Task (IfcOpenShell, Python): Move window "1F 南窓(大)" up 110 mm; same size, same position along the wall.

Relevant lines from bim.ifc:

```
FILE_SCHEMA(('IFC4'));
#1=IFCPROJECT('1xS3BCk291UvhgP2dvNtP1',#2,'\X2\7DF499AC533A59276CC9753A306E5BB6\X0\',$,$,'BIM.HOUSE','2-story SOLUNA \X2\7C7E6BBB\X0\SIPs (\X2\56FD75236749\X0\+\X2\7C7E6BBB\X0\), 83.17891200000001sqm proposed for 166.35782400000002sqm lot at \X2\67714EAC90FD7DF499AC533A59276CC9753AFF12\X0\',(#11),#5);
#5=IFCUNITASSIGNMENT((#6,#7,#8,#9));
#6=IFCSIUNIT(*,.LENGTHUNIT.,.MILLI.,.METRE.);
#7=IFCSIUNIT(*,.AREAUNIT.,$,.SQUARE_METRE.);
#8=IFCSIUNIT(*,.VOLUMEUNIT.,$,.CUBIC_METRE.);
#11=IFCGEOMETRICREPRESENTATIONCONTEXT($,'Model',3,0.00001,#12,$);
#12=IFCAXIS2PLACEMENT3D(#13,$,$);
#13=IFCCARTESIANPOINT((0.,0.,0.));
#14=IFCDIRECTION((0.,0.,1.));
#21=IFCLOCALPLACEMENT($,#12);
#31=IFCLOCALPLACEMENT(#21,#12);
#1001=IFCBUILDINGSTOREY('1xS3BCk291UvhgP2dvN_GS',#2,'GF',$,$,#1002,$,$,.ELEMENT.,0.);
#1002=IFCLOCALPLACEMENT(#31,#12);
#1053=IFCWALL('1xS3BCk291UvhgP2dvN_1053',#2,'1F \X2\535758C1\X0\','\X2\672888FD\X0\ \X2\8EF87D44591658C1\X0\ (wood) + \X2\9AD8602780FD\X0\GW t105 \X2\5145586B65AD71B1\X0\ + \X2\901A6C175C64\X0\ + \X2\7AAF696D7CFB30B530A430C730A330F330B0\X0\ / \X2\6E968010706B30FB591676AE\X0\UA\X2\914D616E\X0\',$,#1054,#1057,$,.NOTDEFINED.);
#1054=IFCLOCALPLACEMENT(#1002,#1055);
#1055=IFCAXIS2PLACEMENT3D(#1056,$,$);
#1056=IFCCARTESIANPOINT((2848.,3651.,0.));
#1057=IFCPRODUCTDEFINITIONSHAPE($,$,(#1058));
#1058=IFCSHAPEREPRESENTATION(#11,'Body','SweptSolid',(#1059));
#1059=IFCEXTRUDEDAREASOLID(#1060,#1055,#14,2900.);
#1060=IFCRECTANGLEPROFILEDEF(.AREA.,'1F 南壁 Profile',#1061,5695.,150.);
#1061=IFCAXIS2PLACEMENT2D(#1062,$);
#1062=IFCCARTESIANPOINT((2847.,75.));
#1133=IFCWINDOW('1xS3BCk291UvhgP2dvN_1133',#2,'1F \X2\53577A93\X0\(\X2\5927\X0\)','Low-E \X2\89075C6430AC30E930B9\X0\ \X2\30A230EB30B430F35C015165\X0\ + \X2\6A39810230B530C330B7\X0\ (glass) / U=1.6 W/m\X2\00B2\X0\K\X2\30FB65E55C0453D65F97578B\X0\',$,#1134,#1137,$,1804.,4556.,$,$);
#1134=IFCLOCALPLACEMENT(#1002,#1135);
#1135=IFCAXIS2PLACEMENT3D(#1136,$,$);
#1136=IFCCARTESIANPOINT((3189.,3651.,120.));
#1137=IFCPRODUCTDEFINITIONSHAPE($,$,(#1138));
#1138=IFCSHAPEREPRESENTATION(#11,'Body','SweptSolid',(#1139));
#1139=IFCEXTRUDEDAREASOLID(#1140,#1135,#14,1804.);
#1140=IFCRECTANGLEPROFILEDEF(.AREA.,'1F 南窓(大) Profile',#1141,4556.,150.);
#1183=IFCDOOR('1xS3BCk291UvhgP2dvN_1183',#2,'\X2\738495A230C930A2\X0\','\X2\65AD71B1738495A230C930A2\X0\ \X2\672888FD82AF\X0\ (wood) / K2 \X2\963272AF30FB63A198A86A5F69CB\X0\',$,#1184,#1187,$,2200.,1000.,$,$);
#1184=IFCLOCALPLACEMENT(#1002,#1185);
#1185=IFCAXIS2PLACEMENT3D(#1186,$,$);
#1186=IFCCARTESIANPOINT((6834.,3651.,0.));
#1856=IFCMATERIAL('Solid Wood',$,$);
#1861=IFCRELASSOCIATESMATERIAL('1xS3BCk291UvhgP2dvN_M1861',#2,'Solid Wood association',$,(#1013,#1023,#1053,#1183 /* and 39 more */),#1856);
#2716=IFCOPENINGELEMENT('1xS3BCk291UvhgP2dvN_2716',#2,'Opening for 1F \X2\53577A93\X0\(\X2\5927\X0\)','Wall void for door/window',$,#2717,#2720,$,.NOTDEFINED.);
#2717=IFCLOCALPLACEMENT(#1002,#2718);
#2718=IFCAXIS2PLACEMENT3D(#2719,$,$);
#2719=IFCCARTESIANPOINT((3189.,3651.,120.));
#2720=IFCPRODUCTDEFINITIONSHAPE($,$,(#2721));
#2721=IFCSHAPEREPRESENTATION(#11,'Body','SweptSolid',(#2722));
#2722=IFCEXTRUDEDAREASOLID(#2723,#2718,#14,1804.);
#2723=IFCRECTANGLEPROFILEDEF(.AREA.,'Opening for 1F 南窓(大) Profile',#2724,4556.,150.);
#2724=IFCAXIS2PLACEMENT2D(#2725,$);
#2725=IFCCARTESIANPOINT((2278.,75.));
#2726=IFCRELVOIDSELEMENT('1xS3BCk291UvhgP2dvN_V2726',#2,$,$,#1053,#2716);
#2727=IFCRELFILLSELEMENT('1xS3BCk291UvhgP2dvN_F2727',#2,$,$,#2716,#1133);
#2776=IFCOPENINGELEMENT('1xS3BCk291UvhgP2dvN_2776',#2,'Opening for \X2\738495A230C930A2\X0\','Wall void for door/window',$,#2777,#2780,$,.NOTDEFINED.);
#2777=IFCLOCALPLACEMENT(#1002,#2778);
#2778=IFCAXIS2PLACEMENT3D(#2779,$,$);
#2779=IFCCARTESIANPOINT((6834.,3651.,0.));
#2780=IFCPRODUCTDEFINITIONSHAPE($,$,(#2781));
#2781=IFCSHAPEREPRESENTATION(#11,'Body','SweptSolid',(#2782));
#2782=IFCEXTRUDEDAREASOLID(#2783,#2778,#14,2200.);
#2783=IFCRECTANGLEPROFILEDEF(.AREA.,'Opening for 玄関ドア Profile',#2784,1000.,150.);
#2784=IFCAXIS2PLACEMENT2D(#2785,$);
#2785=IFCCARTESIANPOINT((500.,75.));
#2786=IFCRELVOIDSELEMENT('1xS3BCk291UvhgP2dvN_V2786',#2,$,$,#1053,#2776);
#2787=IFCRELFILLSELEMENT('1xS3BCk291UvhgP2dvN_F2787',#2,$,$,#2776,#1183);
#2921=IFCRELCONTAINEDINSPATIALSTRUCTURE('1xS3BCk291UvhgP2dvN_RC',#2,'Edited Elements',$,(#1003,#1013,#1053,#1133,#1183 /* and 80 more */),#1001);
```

```python
import numpy as np
import ifcopenshell
import ifcopenshell.api.geometry
import ifcopenshell.util.placement
import ifcopenshell.util.unit

model = ifcopenshell.open("bim.ifc")
unit_scale = ifcopenshell.util.unit.calculate_unit_scale(model)

window = model.by_guid("1xS3BCk291UvhgP2dvN_1133")
opening = window.FillsVoids[0].RelatingOpeningElement
dz = 110.0

shift = np.array([0.0, 0.0, dz])
# The window is not placed relative to its opening, so move both.
for product in (opening, window):
    matrix = ifcopenshell.util.placement.get_local_placement(product.ObjectPlacement)
    matrix[:3, 3] += shift
    ifcopenshell.api.geometry.edit_object_placement(model, product=product, matrix=matrix, is_si=False)

print(f"moved by {dz * unit_scale:+.3f} m")

model.write("bim_rev.ifc")
```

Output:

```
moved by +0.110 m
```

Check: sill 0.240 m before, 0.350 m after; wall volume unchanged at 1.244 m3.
